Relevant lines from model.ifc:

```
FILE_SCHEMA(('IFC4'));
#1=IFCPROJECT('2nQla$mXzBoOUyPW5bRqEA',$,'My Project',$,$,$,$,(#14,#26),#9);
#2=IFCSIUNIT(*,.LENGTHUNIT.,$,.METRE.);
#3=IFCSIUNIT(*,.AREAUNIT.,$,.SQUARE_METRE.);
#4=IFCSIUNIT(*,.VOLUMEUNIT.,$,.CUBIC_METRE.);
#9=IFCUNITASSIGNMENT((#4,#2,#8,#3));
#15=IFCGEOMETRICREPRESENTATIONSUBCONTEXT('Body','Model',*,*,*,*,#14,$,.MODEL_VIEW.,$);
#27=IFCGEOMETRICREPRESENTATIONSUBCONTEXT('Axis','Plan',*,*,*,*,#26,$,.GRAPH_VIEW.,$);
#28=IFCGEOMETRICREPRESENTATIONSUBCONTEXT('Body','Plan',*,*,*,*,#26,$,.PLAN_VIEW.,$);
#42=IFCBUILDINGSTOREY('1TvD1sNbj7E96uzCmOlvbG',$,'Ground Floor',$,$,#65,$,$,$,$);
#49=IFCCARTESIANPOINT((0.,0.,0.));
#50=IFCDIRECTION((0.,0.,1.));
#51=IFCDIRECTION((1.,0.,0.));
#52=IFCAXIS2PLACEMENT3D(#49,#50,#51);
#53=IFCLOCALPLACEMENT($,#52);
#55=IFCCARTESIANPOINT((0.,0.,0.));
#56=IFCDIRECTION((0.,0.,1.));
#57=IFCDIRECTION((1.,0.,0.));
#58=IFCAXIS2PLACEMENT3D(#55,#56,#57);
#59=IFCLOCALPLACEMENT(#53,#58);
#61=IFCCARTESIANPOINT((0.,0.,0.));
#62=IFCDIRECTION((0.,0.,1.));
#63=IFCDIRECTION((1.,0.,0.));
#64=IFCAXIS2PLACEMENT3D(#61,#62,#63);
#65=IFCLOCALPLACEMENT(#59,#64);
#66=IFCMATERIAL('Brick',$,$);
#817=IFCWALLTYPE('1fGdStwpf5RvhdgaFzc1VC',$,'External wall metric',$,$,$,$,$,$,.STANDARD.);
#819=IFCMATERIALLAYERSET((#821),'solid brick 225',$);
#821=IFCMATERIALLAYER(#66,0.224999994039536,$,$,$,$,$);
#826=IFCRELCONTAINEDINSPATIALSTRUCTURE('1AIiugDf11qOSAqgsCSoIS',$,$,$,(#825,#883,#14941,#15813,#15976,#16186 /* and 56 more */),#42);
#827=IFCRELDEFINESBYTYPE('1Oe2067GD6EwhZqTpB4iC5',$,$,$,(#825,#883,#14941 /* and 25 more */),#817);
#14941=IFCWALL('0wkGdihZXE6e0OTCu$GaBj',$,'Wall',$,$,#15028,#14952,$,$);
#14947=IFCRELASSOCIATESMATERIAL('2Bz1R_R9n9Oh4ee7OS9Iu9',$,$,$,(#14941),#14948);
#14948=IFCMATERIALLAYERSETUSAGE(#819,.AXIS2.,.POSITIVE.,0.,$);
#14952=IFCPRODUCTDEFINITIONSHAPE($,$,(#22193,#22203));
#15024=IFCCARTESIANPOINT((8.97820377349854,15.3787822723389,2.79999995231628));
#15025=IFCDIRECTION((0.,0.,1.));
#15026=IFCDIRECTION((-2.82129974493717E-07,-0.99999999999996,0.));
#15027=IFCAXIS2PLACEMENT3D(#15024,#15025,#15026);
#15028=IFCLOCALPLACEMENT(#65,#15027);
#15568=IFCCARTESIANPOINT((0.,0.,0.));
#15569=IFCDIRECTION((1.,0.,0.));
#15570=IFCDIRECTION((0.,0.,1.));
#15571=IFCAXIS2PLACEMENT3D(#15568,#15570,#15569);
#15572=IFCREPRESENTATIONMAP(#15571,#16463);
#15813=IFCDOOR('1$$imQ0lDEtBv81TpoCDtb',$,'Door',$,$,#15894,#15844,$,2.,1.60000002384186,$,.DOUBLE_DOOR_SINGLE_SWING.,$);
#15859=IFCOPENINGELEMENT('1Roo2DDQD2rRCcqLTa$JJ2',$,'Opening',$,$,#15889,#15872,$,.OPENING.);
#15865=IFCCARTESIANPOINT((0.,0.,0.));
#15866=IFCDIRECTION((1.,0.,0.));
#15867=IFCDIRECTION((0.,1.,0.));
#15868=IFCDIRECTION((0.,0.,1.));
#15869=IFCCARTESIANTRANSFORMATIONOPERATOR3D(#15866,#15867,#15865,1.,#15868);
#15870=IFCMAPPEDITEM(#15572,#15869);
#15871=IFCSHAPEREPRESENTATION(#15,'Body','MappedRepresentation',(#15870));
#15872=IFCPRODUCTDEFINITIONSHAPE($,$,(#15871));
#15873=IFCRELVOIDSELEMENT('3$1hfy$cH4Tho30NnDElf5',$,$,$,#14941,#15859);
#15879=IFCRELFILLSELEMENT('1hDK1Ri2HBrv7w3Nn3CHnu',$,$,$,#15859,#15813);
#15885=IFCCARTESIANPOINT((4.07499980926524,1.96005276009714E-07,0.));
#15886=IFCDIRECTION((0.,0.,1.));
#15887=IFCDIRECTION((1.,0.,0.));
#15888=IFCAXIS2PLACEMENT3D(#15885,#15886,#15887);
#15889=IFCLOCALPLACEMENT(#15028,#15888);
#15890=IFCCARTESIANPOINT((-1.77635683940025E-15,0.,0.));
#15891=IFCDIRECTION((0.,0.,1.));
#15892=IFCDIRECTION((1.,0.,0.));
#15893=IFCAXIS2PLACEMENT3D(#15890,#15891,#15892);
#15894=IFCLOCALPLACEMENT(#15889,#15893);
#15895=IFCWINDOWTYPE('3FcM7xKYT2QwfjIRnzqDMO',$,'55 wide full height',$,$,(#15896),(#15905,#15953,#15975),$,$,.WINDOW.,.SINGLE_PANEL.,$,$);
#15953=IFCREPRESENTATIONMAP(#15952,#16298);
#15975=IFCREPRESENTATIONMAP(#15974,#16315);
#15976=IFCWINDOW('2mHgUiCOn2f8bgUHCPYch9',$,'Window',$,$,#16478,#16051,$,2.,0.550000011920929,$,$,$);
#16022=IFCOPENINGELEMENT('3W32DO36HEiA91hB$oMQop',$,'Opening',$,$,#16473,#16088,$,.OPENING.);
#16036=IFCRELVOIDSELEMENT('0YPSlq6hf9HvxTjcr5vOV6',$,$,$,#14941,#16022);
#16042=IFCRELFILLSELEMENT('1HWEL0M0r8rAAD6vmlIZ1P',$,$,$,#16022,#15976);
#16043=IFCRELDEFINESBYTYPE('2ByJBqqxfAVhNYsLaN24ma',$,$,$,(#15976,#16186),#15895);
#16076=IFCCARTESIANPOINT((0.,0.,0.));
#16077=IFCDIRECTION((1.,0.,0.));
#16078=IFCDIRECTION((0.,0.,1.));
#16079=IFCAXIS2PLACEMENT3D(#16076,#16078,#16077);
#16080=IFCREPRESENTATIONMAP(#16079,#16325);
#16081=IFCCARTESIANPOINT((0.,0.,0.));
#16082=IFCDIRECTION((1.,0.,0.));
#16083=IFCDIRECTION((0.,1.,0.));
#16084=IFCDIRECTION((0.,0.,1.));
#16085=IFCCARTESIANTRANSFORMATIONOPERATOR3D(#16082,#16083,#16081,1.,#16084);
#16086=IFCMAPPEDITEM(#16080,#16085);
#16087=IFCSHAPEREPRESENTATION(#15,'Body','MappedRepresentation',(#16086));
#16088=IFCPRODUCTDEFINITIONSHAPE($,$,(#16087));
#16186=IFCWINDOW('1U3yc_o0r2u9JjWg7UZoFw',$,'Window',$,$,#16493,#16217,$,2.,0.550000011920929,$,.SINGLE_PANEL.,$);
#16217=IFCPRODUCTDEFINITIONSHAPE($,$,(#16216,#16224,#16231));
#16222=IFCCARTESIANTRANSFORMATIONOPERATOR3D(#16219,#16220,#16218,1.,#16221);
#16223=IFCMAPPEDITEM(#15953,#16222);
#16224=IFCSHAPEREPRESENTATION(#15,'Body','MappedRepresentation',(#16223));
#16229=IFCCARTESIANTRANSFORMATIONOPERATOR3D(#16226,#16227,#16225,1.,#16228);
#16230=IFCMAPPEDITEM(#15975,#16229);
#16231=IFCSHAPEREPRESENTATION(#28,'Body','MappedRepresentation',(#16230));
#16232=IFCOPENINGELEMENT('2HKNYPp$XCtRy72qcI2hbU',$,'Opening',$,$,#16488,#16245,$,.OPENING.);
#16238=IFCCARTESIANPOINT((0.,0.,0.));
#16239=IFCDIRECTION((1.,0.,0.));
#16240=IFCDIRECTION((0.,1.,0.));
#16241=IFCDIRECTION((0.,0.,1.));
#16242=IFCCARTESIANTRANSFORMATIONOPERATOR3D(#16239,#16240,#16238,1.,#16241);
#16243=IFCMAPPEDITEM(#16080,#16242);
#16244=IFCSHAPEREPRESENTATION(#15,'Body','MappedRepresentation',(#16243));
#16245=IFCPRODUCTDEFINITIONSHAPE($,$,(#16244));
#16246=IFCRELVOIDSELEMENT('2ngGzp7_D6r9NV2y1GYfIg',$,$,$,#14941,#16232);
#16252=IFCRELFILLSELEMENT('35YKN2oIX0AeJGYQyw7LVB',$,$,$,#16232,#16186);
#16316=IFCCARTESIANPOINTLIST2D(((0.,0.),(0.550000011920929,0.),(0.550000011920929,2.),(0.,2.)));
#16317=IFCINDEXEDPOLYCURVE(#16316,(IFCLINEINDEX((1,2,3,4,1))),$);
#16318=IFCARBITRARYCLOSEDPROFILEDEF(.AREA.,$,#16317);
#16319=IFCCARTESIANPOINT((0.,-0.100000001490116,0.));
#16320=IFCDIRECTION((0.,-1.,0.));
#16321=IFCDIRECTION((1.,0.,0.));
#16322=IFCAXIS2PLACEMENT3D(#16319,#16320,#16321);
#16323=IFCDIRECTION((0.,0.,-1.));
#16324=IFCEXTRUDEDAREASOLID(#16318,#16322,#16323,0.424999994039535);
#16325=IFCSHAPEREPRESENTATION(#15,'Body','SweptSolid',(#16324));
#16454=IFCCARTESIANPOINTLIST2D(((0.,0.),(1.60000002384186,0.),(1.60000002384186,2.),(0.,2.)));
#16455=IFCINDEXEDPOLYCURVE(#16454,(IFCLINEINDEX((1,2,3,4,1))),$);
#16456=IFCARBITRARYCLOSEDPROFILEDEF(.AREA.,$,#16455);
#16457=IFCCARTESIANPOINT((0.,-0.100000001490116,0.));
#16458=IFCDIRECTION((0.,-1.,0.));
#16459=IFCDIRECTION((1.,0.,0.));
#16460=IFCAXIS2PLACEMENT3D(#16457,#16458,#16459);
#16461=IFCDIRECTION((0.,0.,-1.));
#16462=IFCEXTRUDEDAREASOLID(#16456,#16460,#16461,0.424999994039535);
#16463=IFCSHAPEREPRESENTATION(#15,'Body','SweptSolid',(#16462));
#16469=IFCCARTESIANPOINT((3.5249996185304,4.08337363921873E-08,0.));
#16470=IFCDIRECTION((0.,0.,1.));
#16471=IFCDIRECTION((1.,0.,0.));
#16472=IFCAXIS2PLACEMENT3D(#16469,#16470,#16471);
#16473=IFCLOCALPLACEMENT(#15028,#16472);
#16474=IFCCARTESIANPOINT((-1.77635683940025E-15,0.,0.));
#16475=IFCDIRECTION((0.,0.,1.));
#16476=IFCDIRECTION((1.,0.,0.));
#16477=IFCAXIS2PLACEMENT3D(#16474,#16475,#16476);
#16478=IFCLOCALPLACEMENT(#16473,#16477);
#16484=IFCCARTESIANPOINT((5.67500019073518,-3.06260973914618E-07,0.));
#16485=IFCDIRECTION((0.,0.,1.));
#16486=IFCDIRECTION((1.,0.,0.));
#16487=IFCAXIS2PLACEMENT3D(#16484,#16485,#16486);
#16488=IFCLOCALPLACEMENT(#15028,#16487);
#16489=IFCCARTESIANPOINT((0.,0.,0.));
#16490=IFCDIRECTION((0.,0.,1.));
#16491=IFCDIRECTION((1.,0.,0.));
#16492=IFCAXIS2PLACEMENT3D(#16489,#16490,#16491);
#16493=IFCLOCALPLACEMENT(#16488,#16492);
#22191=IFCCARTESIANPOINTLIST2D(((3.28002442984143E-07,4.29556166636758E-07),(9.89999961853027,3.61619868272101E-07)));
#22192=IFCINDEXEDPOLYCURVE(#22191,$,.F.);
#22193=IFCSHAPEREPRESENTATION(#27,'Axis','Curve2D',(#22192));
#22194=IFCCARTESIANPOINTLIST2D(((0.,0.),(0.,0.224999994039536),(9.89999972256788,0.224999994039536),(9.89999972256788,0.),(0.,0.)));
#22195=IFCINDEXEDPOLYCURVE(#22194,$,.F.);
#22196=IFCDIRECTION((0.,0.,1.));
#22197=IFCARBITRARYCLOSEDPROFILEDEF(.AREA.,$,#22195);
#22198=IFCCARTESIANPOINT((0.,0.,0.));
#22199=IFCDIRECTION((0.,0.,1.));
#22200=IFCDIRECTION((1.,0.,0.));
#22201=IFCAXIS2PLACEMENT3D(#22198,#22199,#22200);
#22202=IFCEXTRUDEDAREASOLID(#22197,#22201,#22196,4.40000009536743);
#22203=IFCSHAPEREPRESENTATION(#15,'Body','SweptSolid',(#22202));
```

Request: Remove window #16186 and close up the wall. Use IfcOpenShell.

```python
import ifcopenshell
import ifcopenshell.api.feature
import ifcopenshell.api.root
import ifcopenshell.geom
import ifcopenshell.util.shape

model = ifcopenshell.open("model.ifc")
settings = ifcopenshell.geom.settings()


def volume(element):
    """Net volume in cubic metres, openings subtracted."""
    shape = ifcopenshell.geom.create_shape(settings, element)
    return ifcopenshell.util.shape.get_volume(shape.geometry)


window = model.by_id(16186)
opening = window.FillsVoids[0].RelatingOpeningElement
wall = opening.VoidsElements[0].RelatingBuildingElement
before = volume(wall)

ifcopenshell.api.root.remove_product(model, product=window)
ifcopenshell.api.feature.remove_feature(model, feature=opening)

after = volume(wall)

print(f"wall volume {before:.3f} -> {after:.3f} m3")

model.write("model_updated.ifc")
```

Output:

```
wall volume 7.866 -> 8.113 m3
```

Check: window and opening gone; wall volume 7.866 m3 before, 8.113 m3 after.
